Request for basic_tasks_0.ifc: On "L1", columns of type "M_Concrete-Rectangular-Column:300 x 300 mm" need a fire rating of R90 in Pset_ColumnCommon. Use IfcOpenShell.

First a look at what the model holds.

```python
import ifcopenshell
import ifcopenshell.util.element

model = ifcopenshell.open("basic_tasks_0.ifc")
print(model.schema)
storey = next(s for s in model.by_type("IfcBuildingStorey") if s.Name == "L1")
columns = [e for e in ifcopenshell.util.element.get_decomposition(storey) if e.is_a("IfcColumn")]
seen = {}
for e in columns:
    element_type = ifcopenshell.util.element.get_type(e)
    key = (element_type.Name if element_type != e and element_type else None, ifcopenshell.util.element.get_pset(e, "Pset_ColumnCommon", "FireRating"))
    seen[key] = seen.get(key, 0) + 1
for (name, value), count in sorted(seen.items(), key=str):
    print(count, "x", name, "|", value)
```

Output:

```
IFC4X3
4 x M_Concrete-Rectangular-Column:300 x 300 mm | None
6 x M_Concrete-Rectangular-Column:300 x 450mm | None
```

```python
import ifcopenshell
import ifcopenshell.api.pset
import ifcopenshell.util.element

model = ifcopenshell.open("basic_tasks_0.ifc")

storey = next(s for s in model.by_type("IfcBuildingStorey") if s.Name == "L1")
columns = [e for e in ifcopenshell.util.element.get_decomposition(storey) if e.is_a("IfcColumn")]

count = 0
for e in columns:
    element_type = ifcopenshell.util.element.get_type(e)
    if element_type in (None, e) or element_type.Name != "M_Concrete-Rectangular-Column:300 x 300 mm":
        continue
    # add_pset returns the element's existing set when there is one.
    pset = ifcopenshell.api.pset.add_pset(model, product=e, name="Pset_ColumnCommon")
    ifcopenshell.api.pset.edit_pset(model, pset=pset, properties={"FireRating": "R90"})
    count += 1

print(count, "columns updated")

model.write("basic_tasks_0-out.ifc")
```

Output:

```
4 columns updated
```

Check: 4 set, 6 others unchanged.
